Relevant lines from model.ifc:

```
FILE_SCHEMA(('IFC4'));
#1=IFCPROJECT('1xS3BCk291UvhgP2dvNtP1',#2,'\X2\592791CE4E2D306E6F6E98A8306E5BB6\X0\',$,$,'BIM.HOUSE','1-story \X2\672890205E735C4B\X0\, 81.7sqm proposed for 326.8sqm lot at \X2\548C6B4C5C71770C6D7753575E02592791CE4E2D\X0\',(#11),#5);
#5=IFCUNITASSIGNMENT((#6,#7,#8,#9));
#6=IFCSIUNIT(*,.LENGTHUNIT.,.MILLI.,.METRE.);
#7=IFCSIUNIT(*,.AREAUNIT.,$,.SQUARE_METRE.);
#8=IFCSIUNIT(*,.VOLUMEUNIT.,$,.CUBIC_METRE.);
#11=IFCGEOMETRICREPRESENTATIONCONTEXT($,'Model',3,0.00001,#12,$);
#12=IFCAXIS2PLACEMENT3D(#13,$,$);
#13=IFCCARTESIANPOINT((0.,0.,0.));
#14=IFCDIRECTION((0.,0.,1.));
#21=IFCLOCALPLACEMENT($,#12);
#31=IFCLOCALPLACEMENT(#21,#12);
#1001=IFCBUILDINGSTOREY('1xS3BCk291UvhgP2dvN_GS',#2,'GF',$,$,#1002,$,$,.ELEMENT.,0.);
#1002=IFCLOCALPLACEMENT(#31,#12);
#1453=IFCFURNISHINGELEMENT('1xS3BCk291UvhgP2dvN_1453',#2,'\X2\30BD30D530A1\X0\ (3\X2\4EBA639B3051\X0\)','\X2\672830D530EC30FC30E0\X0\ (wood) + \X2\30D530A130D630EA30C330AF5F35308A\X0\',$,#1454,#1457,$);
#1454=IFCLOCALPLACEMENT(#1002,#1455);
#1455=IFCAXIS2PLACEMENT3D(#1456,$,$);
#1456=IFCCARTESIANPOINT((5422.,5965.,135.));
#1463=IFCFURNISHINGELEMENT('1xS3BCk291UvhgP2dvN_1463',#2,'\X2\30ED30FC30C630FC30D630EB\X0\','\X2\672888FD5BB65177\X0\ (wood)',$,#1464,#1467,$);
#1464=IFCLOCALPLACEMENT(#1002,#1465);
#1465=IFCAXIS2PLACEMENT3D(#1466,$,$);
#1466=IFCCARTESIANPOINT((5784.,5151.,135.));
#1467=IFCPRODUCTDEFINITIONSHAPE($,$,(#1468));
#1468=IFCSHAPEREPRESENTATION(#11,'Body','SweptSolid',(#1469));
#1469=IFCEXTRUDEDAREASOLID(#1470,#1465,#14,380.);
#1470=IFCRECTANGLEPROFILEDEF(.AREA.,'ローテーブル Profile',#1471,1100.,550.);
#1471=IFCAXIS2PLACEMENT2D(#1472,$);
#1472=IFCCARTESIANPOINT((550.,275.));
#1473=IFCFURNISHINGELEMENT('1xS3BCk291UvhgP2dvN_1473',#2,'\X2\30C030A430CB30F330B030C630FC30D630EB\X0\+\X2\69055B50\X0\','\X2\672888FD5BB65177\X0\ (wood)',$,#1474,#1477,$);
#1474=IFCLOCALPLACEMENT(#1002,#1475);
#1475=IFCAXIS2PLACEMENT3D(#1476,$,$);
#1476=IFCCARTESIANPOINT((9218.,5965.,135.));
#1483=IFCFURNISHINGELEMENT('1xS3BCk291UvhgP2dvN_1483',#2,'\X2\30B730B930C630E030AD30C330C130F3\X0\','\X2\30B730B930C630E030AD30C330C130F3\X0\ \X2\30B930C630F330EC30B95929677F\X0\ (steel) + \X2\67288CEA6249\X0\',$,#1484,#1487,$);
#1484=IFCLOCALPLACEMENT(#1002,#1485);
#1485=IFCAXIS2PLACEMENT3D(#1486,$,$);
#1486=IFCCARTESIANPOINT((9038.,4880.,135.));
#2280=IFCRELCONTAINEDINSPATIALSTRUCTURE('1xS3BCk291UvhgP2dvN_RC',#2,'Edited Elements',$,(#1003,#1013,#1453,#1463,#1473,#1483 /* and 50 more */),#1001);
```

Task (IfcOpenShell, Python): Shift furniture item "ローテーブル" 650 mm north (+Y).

```python
import ifcopenshell
import ifcopenshell.api.geometry
import ifcopenshell.util.placement
import ifcopenshell.util.unit

model = ifcopenshell.open("model.ifc")
unit_scale = ifcopenshell.util.unit.calculate_unit_scale(model)

item = model.by_guid("1xS3BCk291UvhgP2dvN_1463")
matrix = ifcopenshell.util.placement.get_local_placement(item.ObjectPlacement)
matrix[1, 3] += 0.65 / unit_scale
ifcopenshell.api.geometry.edit_object_placement(model, product=item, matrix=matrix, is_si=False)

print(ifcopenshell.util.placement.get_local_placement(item.ObjectPlacement).round(3) + 0.0)

model.write("model_updated.ifc")
```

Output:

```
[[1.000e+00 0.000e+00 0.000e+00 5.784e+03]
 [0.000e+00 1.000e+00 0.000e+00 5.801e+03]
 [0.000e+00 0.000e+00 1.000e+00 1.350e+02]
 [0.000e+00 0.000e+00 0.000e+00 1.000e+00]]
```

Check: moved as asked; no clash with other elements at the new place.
